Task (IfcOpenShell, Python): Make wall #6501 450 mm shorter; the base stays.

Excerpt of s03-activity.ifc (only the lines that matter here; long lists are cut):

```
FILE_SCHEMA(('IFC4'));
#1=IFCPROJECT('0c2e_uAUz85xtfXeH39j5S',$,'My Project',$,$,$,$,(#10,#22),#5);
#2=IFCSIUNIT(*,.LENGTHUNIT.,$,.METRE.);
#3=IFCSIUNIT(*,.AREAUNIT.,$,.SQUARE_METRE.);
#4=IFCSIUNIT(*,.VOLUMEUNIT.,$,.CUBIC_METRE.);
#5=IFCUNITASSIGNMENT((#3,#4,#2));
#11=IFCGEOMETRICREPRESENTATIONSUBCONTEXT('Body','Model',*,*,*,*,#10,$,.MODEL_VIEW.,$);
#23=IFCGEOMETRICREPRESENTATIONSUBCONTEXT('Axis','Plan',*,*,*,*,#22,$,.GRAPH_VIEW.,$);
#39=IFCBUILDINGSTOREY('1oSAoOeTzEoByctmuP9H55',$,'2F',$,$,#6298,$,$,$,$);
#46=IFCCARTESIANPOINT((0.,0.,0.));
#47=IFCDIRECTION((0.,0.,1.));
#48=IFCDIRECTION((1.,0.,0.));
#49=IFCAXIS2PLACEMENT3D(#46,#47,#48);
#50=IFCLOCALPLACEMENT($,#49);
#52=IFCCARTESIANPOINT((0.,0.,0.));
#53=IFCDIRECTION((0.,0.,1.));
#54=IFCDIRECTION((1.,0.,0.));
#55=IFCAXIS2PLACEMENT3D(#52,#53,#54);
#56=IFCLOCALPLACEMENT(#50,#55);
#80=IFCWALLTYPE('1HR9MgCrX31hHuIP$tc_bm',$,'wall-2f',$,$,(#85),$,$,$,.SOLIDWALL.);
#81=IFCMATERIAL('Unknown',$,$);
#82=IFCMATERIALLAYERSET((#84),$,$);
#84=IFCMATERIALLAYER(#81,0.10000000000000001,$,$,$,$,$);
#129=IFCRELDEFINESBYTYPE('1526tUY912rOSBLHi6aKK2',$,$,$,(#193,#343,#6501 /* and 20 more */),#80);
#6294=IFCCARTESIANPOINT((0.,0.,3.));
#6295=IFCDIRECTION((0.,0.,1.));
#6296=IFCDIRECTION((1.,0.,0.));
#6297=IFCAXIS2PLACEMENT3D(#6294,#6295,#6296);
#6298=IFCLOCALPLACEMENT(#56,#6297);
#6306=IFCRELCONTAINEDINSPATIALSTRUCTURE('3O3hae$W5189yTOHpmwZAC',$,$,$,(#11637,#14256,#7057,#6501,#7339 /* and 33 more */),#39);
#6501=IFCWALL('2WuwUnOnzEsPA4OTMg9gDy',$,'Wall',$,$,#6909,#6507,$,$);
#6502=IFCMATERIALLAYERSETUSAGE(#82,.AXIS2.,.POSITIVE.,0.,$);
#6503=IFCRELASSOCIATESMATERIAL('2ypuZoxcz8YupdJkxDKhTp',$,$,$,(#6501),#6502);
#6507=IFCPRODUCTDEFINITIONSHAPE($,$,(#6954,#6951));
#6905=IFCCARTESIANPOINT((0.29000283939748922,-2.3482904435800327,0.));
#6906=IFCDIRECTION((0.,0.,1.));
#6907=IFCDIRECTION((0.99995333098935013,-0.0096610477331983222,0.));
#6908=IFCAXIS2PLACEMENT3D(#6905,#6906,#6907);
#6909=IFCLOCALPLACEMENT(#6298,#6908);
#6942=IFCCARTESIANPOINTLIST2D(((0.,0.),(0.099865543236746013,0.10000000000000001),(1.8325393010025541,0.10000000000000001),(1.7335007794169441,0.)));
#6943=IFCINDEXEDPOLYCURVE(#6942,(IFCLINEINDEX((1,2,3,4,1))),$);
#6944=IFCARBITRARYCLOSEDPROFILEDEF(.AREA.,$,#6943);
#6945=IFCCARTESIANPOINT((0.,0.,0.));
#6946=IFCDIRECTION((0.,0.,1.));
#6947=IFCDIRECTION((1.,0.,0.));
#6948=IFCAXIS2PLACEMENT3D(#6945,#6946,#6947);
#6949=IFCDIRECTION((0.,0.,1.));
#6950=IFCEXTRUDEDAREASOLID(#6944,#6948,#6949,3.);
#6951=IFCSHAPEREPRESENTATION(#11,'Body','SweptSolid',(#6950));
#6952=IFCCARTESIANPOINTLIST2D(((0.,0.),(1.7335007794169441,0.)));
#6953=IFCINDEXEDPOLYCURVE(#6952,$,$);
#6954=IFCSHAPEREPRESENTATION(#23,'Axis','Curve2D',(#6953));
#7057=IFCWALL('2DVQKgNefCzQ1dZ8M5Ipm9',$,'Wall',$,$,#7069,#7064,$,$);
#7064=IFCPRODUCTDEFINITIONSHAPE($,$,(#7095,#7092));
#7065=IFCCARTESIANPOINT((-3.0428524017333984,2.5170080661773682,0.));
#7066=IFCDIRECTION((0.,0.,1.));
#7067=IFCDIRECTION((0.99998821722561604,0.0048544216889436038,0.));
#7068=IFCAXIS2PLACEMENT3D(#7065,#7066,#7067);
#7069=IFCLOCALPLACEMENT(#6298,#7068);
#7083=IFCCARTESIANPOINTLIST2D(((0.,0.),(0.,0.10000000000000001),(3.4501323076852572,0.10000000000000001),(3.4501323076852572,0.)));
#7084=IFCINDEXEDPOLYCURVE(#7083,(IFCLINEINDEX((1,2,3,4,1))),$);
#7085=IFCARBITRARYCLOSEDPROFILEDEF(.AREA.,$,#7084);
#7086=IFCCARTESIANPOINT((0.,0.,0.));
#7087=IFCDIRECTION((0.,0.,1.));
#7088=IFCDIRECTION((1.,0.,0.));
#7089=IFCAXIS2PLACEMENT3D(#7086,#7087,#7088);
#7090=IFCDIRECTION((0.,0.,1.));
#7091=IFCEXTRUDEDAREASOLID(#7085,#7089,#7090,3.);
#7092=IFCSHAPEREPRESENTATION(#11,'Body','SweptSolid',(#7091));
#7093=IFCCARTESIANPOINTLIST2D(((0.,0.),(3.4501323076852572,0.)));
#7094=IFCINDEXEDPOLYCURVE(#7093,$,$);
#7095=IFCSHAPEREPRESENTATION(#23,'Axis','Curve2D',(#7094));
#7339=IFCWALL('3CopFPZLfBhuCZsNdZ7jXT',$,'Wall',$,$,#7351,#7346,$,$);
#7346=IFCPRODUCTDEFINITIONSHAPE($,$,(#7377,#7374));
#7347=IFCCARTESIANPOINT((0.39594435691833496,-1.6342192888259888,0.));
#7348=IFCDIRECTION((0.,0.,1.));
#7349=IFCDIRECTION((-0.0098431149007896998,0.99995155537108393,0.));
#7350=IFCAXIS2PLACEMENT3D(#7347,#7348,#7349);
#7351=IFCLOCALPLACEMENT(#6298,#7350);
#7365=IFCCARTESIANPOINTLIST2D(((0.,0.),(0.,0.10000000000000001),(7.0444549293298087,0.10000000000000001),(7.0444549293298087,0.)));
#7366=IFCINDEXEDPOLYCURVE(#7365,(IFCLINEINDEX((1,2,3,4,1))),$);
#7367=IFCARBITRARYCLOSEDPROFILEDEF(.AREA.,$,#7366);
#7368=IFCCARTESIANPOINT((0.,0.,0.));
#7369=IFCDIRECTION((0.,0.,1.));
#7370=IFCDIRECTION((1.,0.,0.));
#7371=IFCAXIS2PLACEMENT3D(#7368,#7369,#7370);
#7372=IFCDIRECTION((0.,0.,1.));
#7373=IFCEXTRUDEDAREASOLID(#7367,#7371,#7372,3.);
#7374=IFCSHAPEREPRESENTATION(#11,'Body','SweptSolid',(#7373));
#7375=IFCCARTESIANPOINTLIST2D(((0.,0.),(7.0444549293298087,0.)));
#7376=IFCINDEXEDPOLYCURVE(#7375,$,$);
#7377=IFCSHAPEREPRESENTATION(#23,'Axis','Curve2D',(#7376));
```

```python
import ifcopenshell
import ifcopenshell.geom
import ifcopenshell.util.representation
import ifcopenshell.util.shape
import ifcopenshell.util.unit

model = ifcopenshell.open("s03-activity.ifc")
unit_scale = ifcopenshell.util.unit.calculate_unit_scale(model)
settings = ifcopenshell.geom.settings()


def volume(element):
    """Net volume in cubic metres, openings subtracted."""
    shape = ifcopenshell.geom.create_shape(settings, element)
    return ifcopenshell.util.shape.get_volume(shape.geometry)


wall = model.by_id(6501)
before = volume(wall)

body = ifcopenshell.util.representation.get_representation(wall, "Model", "Body")
solid = body.Items[0]
old_height = solid.Depth
solid.Depth -= 0.45 / unit_scale
after = volume(wall)

print(f"height {old_height:g} -> {solid.Depth:g}, volume {before:.3f} -> {after:.3f} m3")

model.write("s03-activity_v2.ifc")
```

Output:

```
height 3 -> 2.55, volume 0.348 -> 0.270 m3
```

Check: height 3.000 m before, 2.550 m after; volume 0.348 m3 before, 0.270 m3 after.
